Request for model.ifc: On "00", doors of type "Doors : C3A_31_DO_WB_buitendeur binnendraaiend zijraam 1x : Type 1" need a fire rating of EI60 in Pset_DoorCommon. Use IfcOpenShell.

First a look at what the model holds.

```python
import ifcopenshell
import ifcopenshell.util.element

model = ifcopenshell.open("model.ifc")
print(model.schema)
storey = next(s for s in model.by_type("IfcBuildingStorey") if s.Name == "00")
doors = [e for e in ifcopenshell.util.element.get_decomposition(storey) if e.is_a("IfcDoor")]
seen = {}
for e in doors:
    element_type = ifcopenshell.util.element.get_type(e)
    key = (element_type.Name if element_type != e and element_type else None, ifcopenshell.util.element.get_pset(e, "Pset_DoorCommon", "FireRating"))
    seen[key] = seen.get(key, 0) + 1
for (name, value), count in sorted(seen.items(), key=str):
    print(count, "x", name, "|", value)
```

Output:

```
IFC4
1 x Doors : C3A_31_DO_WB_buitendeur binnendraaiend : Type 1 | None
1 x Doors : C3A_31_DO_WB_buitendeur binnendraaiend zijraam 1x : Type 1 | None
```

```python
import ifcopenshell
import ifcopenshell.api.pset
import ifcopenshell.util.element

model = ifcopenshell.open("model.ifc")

storey = next(s for s in model.by_type("IfcBuildingStorey") if s.Name == "00")
doors = [e for e in ifcopenshell.util.element.get_decomposition(storey) if e.is_a("IfcDoor")]

count = 0
for e in doors:
    element_type = ifcopenshell.util.element.get_type(e)
    if element_type in (None, e) or element_type.Name != "Doors : C3A_31_DO_WB_buitendeur binnendraaiend zijraam 1x : Type 1":
        continue
    # add_pset returns the element's existing set when there is one.
    pset = ifcopenshell.api.pset.add_pset(model, product=e, name="Pset_DoorCommon")
    ifcopenshell.api.pset.edit_pset(model, pset=pset, properties={"FireRating": "EI60"})
    count += 1

print(count, "doors updated")

model.write("model_updated.ifc")
```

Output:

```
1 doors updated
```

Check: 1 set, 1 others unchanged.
